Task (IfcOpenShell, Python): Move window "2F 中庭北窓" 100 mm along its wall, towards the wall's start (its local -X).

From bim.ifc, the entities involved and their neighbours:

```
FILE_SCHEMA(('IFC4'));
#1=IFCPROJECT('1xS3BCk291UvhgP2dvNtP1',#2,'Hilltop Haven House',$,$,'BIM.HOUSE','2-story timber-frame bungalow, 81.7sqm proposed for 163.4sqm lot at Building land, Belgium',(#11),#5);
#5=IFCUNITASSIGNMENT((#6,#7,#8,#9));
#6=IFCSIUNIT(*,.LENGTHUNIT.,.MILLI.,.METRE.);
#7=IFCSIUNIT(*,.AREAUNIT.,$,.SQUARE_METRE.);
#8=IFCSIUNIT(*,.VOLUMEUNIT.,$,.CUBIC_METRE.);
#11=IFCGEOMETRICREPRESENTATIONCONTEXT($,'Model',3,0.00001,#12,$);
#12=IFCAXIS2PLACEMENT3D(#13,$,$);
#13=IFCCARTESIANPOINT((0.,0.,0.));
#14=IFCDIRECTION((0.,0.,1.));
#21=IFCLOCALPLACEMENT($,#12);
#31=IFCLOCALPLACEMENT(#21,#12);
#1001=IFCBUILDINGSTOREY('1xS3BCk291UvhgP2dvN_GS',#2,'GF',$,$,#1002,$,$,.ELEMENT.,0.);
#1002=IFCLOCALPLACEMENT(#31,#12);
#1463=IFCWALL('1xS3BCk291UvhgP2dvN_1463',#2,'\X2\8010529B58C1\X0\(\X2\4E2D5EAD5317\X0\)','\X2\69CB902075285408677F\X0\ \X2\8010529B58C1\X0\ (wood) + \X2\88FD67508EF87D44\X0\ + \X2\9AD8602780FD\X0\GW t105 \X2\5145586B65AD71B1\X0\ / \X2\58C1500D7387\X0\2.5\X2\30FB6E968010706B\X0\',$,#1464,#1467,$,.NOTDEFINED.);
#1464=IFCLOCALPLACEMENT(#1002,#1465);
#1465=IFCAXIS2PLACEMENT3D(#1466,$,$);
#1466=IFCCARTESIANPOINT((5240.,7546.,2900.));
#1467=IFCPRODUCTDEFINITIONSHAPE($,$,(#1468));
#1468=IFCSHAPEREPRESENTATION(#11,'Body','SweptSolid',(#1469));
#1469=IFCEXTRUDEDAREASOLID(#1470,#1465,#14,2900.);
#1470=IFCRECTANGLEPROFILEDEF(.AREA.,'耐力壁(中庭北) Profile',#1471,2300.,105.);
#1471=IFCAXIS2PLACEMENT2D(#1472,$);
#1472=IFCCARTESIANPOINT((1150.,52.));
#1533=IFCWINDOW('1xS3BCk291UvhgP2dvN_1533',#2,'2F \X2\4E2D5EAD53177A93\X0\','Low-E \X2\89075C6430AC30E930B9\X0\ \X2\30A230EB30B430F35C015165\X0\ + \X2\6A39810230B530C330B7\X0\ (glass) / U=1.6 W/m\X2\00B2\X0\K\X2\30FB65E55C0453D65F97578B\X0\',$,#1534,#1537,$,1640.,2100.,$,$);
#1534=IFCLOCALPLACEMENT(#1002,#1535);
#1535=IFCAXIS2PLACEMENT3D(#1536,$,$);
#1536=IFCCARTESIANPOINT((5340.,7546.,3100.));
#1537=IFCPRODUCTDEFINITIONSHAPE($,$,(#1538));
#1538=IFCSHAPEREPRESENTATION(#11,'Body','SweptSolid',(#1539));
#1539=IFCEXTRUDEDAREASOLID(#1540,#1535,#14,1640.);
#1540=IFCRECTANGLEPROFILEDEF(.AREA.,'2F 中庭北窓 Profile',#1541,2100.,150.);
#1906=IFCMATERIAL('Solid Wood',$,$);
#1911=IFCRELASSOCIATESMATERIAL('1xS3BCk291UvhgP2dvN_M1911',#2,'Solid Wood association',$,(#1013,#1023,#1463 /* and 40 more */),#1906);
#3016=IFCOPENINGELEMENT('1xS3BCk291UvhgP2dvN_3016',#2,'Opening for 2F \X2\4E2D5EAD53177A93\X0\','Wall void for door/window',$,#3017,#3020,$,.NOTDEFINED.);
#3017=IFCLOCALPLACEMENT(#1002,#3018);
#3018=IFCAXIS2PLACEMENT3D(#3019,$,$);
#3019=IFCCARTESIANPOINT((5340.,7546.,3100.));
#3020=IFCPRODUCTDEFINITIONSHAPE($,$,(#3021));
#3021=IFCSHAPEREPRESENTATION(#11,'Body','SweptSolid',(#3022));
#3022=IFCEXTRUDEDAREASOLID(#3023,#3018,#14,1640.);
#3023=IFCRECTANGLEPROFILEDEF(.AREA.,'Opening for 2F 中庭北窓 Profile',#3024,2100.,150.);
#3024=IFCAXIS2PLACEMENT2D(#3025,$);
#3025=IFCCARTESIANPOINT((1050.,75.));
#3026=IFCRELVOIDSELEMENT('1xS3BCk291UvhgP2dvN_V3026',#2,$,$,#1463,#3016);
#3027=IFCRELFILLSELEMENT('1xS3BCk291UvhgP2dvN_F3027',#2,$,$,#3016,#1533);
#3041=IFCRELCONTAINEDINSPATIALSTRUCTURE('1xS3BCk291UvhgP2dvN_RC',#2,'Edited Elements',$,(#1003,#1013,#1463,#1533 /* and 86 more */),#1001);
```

```python
import ifcopenshell
import ifcopenshell.api.geometry
import ifcopenshell.util.placement
import ifcopenshell.util.unit

model = ifcopenshell.open("bim.ifc")
unit_scale = ifcopenshell.util.unit.calculate_unit_scale(model)

window = model.by_guid("1xS3BCk291UvhgP2dvN_1533")
opening = window.FillsVoids[0].RelatingOpeningElement
wall = opening.VoidsElements[0].RelatingBuildingElement

wall_matrix = ifcopenshell.util.placement.get_local_placement(wall.ObjectPlacement)
shift = wall_matrix[:3, 0] * -0.1 / unit_scale
before = ifcopenshell.util.placement.get_local_placement(window.ObjectPlacement)[:3, 3].copy()

# The window is not placed relative to its opening, so move both.
for product in (opening, window):
    matrix = ifcopenshell.util.placement.get_local_placement(product.ObjectPlacement)
    matrix[:3, 3] += shift
    ifcopenshell.api.geometry.edit_object_placement(model, product=product, matrix=matrix, is_si=False)

after = ifcopenshell.util.placement.get_local_placement(window.ObjectPlacement)[:3, 3]
print("window moved by", (after - before).round(3) + 0.0)

model.write("bim-out.ifc")
```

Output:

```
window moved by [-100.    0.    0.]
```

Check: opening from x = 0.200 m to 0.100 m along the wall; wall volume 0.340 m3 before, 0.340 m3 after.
